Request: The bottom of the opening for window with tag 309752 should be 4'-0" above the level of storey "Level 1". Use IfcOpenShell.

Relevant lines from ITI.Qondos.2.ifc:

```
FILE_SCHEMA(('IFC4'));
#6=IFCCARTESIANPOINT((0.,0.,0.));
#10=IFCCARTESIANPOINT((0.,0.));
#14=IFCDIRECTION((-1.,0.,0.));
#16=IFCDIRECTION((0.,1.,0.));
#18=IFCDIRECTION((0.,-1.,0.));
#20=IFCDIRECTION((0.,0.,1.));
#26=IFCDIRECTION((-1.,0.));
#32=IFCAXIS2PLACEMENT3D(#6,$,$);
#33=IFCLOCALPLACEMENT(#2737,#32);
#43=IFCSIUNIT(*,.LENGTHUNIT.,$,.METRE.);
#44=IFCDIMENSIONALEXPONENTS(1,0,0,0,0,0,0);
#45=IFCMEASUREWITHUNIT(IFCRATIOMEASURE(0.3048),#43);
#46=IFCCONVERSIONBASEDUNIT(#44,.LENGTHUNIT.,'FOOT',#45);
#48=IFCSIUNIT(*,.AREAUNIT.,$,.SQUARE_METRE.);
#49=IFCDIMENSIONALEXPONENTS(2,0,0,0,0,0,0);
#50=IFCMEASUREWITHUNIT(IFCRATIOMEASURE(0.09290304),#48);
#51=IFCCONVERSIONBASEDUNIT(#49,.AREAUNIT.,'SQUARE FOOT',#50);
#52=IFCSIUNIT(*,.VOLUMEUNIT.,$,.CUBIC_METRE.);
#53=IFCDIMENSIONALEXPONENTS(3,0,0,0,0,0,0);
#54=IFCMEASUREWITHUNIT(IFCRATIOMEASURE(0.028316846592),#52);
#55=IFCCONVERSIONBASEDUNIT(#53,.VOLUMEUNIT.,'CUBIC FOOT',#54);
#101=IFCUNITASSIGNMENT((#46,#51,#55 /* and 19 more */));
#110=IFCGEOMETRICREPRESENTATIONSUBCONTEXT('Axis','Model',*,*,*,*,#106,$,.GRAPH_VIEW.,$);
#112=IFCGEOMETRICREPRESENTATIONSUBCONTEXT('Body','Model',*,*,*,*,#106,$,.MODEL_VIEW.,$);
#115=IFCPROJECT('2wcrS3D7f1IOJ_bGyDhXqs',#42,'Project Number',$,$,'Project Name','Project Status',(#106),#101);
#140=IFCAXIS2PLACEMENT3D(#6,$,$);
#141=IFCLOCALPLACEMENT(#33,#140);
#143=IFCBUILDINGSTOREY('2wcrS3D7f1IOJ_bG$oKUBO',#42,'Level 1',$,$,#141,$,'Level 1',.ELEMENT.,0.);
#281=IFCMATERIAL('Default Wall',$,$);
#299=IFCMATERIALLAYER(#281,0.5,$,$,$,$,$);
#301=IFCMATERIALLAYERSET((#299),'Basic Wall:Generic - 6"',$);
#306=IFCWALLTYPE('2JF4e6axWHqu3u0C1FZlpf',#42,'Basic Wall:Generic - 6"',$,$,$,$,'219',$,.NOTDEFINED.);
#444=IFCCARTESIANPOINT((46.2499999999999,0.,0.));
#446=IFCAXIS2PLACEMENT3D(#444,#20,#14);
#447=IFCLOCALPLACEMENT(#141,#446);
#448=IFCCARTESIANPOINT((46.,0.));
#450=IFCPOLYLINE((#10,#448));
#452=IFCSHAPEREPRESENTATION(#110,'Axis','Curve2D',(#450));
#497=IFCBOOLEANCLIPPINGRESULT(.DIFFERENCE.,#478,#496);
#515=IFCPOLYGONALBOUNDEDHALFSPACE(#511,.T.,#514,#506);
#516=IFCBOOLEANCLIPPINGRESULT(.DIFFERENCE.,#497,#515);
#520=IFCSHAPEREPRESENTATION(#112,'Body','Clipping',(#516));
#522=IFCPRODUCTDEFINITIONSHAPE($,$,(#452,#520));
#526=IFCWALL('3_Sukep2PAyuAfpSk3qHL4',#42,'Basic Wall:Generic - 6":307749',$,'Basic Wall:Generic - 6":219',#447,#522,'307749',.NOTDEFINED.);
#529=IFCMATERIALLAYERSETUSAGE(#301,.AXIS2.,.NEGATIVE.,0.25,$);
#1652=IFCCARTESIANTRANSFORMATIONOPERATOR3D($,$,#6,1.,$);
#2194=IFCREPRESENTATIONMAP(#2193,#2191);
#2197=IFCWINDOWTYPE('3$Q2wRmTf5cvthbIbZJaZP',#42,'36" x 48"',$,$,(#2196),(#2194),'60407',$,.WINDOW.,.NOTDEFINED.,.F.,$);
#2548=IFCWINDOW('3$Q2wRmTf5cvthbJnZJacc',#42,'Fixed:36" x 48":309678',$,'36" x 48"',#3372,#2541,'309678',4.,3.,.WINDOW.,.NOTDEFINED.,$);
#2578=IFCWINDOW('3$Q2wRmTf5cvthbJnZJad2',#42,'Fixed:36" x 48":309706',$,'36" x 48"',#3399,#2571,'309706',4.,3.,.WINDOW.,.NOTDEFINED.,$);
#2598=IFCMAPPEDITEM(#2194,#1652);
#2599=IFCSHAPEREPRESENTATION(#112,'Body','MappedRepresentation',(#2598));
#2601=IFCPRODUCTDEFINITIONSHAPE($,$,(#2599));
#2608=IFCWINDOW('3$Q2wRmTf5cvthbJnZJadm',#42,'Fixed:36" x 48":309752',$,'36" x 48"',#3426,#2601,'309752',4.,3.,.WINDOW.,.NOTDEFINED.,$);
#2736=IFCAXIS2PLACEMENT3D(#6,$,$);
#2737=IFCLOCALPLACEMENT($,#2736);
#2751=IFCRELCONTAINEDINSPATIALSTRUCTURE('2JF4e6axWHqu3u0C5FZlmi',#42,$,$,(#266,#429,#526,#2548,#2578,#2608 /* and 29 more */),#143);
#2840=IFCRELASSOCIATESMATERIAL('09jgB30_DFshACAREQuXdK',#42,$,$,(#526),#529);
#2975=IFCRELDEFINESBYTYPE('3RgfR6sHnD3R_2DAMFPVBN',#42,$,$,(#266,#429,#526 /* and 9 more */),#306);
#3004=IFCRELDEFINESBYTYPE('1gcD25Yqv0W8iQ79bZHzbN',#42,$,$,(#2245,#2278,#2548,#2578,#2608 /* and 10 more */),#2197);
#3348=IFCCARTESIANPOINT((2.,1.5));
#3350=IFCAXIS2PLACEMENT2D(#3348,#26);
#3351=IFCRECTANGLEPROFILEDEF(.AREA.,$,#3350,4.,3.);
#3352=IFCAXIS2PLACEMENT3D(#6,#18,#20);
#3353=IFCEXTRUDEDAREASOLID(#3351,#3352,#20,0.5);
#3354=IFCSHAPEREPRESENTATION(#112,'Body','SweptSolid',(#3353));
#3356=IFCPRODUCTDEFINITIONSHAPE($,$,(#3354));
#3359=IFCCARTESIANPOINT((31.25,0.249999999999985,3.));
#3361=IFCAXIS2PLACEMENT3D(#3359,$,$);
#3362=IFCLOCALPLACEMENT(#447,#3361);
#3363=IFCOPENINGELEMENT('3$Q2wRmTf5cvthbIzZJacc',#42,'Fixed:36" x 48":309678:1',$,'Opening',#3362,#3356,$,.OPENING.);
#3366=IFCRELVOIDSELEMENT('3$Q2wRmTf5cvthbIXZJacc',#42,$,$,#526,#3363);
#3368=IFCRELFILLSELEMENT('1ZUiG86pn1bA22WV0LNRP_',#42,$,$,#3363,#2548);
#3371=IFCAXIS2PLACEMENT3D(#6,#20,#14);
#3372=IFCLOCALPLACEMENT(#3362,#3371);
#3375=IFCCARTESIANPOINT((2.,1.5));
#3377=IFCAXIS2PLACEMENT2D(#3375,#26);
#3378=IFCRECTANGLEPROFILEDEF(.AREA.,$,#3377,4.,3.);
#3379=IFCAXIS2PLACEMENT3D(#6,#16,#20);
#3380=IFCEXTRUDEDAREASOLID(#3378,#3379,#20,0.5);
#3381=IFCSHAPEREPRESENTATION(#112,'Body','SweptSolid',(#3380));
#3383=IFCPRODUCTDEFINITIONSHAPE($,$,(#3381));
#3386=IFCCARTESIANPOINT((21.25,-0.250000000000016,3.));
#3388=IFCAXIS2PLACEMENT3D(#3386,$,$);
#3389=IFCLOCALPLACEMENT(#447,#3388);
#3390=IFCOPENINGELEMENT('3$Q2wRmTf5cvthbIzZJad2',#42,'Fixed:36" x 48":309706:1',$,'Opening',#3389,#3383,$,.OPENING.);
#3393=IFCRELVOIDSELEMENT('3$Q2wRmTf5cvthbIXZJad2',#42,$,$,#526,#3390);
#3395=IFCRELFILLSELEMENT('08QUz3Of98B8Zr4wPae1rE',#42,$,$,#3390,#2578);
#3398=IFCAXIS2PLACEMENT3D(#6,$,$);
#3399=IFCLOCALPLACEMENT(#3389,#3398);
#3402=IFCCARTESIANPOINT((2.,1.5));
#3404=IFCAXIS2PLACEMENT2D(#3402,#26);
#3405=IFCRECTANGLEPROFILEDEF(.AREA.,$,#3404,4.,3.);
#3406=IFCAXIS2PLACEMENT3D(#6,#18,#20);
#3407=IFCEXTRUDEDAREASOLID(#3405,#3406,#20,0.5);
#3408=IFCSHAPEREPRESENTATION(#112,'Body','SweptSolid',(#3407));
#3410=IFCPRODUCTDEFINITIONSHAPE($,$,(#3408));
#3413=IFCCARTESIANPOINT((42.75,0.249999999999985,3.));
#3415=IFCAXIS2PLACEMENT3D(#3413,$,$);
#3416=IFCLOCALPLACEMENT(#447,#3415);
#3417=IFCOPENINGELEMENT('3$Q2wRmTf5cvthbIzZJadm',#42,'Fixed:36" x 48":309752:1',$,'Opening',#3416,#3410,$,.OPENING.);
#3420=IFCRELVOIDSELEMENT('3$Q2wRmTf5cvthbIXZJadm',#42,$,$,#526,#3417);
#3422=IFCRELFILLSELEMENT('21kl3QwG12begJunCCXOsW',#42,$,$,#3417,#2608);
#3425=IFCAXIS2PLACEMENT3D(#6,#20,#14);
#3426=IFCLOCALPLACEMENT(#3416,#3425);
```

```python
import numpy as np
import ifcopenshell
import ifcopenshell.api.geometry
import ifcopenshell.geom
import ifcopenshell.util.element
import ifcopenshell.util.placement
import ifcopenshell.util.shape
import ifcopenshell.util.unit

model = ifcopenshell.open("ITI.Qondos.2.ifc")
unit_scale = ifcopenshell.util.unit.calculate_unit_scale(model)

window = model.by_id(2608)
opening = window.FillsVoids[0].RelatingOpeningElement
storey = ifcopenshell.util.element.get_container(window, ifc_class="IfcBuildingStorey")
level = ifcopenshell.util.placement.get_local_placement(storey.ObjectPlacement)[2, 3]

# The opening's origin need not be at the sill, so measure its lowest point.
shape = ifcopenshell.geom.create_shape(ifcopenshell.geom.settings(), opening)
bottom = ifcopenshell.util.shape.get_shape_bottom_elevation(shape, shape.geometry) / unit_scale
dz = level + 48 * 0.0254 / unit_scale - bottom

shift = np.array([0.0, 0.0, dz])
# The window is placed relative to its opening, so it follows when the opening moves.
matrix = ifcopenshell.util.placement.get_local_placement(opening.ObjectPlacement)
matrix[:3, 3] += shift
ifcopenshell.api.geometry.edit_object_placement(
    model, product=opening, matrix=matrix, is_si=False, should_transform_children=True
)

print(f"moved by {dz * unit_scale:+.3f} m")

model.write("ITI.Qondos.2-out.ifc")
```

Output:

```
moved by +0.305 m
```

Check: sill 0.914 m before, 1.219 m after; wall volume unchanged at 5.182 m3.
